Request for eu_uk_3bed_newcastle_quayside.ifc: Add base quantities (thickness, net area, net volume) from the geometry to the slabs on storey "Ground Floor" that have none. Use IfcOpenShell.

First a look at what the model holds.

```python
import ifcopenshell
import ifcopenshell.util.element
import ifcopenshell.util.unit

model = ifcopenshell.open("eu_uk_3bed_newcastle_quayside.ifc")
print(model.schema)
for unit_type in ("LENGTHUNIT", "AREAUNIT", "VOLUMEUNIT"):
    print(unit_type, ifcopenshell.util.unit.calculate_unit_scale(model, unit_type))
storey = next(s for s in model.by_type("IfcBuildingStorey") if s.Name == "Ground Floor")
slabs = [e for e in ifcopenshell.util.element.get_decomposition(storey) if e.is_a("IfcSlab")]
for e in sorted(slabs, key=lambda e: e.id()):
    print(e.id(), e.is_a(), e.Name, list(ifcopenshell.util.element.get_psets(e, qtos_only=True)), sep=" | ")
```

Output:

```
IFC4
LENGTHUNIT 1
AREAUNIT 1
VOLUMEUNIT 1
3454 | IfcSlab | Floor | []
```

```python
import ifcopenshell
import ifcopenshell.api.pset
import ifcopenshell.geom
import ifcopenshell.util.element
import ifcopenshell.util.shape
import ifcopenshell.util.unit

model = ifcopenshell.open("eu_uk_3bed_newcastle_quayside.ifc")
unit_scale = ifcopenshell.util.unit.calculate_unit_scale(model)
area_scale = ifcopenshell.util.unit.calculate_unit_scale(model, "AREAUNIT")
volume_scale = ifcopenshell.util.unit.calculate_unit_scale(model, "VOLUMEUNIT")
settings = ifcopenshell.geom.settings()

storey = next(s for s in model.by_type("IfcBuildingStorey") if s.Name == "Ground Floor")
slabs = [e for e in ifcopenshell.util.element.get_decomposition(storey) if e.is_a("IfcSlab")]

for e in sorted(slabs, key=lambda e: e.id()):
    if ifcopenshell.util.element.get_psets(e, qtos_only=True, should_inherit=False):
        continue
    # Geometry comes back in metres, in the element's own axes.
    shape = ifcopenshell.geom.create_shape(settings, e)
    values = {
        "Width": ifcopenshell.util.shape.get_z(shape.geometry) / unit_scale,
        "NetArea": ifcopenshell.util.shape.get_footprint_area(shape.geometry) / area_scale,
        "NetVolume": ifcopenshell.util.shape.get_volume(shape.geometry) / volume_scale,
    }
    qto = ifcopenshell.api.pset.add_qto(model, product=e, name="Qto_SlabBaseQuantities")
    ifcopenshell.api.pset.edit_qto(model, qto=qto, properties=values)
    print(e.id(), {k: round(v, 3) for k, v in values.items()})

model.write("eu_uk_3bed_newcastle_quayside-out.ifc")
```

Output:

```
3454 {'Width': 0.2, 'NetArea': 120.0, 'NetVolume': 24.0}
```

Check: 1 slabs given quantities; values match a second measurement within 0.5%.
